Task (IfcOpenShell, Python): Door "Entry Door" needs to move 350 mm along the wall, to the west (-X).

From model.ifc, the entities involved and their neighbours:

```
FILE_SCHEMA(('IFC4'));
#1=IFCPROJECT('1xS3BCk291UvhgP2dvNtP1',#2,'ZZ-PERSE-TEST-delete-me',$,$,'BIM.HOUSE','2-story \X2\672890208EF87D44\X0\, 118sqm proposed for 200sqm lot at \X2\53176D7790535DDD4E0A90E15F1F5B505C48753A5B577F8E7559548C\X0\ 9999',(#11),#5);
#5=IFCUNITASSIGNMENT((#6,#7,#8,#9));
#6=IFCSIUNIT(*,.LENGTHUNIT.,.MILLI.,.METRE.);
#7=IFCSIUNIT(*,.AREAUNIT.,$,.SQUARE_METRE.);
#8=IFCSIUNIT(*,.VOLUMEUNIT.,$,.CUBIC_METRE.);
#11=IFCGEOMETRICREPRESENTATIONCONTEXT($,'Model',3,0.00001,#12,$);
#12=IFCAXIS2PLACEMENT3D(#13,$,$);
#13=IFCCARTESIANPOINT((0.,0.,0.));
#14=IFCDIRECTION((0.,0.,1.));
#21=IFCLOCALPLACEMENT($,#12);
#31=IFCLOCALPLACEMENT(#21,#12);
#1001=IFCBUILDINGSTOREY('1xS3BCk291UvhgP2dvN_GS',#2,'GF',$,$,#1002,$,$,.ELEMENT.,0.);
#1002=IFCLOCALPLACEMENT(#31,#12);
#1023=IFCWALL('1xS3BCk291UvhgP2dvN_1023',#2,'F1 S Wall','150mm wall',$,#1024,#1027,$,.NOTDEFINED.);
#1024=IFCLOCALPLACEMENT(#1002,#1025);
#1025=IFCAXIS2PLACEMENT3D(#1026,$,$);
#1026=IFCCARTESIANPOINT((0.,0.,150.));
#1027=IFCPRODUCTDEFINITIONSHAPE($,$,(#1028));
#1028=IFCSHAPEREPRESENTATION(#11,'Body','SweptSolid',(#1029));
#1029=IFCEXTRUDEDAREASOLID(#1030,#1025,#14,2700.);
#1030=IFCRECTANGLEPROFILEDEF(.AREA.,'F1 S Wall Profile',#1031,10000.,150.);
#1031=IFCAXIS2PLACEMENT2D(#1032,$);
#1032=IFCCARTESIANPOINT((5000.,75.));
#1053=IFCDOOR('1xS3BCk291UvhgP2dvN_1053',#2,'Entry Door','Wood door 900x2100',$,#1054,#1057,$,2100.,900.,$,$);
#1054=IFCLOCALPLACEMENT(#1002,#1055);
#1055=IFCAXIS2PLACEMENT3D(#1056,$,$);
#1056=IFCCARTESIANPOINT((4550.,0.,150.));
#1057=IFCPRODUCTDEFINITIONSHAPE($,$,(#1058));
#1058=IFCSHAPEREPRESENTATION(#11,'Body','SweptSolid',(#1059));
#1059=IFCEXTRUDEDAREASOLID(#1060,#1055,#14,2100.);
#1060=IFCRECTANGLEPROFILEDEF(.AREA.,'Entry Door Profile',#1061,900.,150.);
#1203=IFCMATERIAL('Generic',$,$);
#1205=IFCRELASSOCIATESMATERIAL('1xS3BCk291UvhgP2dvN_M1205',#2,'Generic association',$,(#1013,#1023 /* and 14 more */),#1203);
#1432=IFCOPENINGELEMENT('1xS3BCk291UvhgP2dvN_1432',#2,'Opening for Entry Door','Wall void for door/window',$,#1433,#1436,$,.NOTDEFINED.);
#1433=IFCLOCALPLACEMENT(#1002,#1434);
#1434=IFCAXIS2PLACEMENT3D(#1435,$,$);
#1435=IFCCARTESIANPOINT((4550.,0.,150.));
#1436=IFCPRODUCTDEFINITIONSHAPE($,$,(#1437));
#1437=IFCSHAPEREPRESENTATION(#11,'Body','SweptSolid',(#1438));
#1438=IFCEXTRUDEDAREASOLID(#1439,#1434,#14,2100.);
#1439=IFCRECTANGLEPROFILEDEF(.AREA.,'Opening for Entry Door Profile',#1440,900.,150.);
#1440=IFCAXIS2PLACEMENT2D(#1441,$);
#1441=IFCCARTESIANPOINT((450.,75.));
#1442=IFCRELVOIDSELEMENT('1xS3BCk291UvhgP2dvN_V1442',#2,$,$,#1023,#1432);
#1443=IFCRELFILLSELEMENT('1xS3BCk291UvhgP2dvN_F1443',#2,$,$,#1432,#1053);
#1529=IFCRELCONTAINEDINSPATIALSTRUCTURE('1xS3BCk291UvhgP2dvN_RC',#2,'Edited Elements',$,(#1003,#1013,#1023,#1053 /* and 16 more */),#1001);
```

```python
import ifcopenshell
import ifcopenshell.api.geometry
import ifcopenshell.util.placement

model = ifcopenshell.open("model.ifc")

door = model.by_guid("1xS3BCk291UvhgP2dvN_1053")
opening = door.FillsVoids[0].RelatingOpeningElement
wall = opening.VoidsElements[0].RelatingBuildingElement

wall_matrix = ifcopenshell.util.placement.get_local_placement(wall.ObjectPlacement)
shift = wall_matrix[:3, 0] * -350.0
before = ifcopenshell.util.placement.get_local_placement(door.ObjectPlacement)[:3, 3].copy()

# The door is not placed relative to its opening, so move both.
for product in (opening, door):
    matrix = ifcopenshell.util.placement.get_local_placement(product.ObjectPlacement)
    matrix[:3, 3] += shift
    ifcopenshell.api.geometry.edit_object_placement(model, product=product, matrix=matrix, is_si=False)

after = ifcopenshell.util.placement.get_local_placement(door.ObjectPlacement)[:3, 3]
print("door moved by", (after - before).round(3) + 0.0)

model.write("model_rev.ifc")
```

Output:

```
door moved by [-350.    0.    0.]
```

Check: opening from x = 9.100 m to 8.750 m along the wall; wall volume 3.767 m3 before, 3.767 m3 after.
